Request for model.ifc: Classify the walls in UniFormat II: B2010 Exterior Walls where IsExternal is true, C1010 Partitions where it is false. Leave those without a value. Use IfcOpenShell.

First a look at what the model holds.

```python
import ifcopenshell
import ifcopenshell.util.element

model = ifcopenshell.open("model.ifc")
print(model.schema)
print("classifications:", [c.Name for c in model.by_type("IfcClassification")])
values = [ifcopenshell.util.element.get_pset(e, "Pset_WallCommon", "IsExternal") for e in model.by_type("IfcWall")]
for value in (True, False, None):
    print("IsExternal", value, values.count(value))
```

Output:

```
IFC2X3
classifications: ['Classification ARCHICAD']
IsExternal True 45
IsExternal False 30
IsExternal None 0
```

```python
import ifcopenshell
import ifcopenshell.api.classification
import ifcopenshell.util.element

model = ifcopenshell.open("model.ifc")

# IFC2X3 requires Source and Edition and has no link from the project to the system.
system = model.create_entity("IfcClassification", Source="ASTM", Edition="E1557", Name="UniFormat II")

walls = model.by_type("IfcWall")
external = {e: ifcopenshell.util.element.get_pset(e, "Pset_WallCommon", "IsExternal") for e in walls}
for flag, code, name in ((True, "B2010", "Exterior Walls"), (False, "C1010", "Partitions")):
    products = [e for e in walls if external[e] is flag]
    ifcopenshell.api.classification.add_reference(
        model, products=products, classification=system, identification=code, name=name
    )
    print(code, len(products))

model.write("model_rev.ifc")
```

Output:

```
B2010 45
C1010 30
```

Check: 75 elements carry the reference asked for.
